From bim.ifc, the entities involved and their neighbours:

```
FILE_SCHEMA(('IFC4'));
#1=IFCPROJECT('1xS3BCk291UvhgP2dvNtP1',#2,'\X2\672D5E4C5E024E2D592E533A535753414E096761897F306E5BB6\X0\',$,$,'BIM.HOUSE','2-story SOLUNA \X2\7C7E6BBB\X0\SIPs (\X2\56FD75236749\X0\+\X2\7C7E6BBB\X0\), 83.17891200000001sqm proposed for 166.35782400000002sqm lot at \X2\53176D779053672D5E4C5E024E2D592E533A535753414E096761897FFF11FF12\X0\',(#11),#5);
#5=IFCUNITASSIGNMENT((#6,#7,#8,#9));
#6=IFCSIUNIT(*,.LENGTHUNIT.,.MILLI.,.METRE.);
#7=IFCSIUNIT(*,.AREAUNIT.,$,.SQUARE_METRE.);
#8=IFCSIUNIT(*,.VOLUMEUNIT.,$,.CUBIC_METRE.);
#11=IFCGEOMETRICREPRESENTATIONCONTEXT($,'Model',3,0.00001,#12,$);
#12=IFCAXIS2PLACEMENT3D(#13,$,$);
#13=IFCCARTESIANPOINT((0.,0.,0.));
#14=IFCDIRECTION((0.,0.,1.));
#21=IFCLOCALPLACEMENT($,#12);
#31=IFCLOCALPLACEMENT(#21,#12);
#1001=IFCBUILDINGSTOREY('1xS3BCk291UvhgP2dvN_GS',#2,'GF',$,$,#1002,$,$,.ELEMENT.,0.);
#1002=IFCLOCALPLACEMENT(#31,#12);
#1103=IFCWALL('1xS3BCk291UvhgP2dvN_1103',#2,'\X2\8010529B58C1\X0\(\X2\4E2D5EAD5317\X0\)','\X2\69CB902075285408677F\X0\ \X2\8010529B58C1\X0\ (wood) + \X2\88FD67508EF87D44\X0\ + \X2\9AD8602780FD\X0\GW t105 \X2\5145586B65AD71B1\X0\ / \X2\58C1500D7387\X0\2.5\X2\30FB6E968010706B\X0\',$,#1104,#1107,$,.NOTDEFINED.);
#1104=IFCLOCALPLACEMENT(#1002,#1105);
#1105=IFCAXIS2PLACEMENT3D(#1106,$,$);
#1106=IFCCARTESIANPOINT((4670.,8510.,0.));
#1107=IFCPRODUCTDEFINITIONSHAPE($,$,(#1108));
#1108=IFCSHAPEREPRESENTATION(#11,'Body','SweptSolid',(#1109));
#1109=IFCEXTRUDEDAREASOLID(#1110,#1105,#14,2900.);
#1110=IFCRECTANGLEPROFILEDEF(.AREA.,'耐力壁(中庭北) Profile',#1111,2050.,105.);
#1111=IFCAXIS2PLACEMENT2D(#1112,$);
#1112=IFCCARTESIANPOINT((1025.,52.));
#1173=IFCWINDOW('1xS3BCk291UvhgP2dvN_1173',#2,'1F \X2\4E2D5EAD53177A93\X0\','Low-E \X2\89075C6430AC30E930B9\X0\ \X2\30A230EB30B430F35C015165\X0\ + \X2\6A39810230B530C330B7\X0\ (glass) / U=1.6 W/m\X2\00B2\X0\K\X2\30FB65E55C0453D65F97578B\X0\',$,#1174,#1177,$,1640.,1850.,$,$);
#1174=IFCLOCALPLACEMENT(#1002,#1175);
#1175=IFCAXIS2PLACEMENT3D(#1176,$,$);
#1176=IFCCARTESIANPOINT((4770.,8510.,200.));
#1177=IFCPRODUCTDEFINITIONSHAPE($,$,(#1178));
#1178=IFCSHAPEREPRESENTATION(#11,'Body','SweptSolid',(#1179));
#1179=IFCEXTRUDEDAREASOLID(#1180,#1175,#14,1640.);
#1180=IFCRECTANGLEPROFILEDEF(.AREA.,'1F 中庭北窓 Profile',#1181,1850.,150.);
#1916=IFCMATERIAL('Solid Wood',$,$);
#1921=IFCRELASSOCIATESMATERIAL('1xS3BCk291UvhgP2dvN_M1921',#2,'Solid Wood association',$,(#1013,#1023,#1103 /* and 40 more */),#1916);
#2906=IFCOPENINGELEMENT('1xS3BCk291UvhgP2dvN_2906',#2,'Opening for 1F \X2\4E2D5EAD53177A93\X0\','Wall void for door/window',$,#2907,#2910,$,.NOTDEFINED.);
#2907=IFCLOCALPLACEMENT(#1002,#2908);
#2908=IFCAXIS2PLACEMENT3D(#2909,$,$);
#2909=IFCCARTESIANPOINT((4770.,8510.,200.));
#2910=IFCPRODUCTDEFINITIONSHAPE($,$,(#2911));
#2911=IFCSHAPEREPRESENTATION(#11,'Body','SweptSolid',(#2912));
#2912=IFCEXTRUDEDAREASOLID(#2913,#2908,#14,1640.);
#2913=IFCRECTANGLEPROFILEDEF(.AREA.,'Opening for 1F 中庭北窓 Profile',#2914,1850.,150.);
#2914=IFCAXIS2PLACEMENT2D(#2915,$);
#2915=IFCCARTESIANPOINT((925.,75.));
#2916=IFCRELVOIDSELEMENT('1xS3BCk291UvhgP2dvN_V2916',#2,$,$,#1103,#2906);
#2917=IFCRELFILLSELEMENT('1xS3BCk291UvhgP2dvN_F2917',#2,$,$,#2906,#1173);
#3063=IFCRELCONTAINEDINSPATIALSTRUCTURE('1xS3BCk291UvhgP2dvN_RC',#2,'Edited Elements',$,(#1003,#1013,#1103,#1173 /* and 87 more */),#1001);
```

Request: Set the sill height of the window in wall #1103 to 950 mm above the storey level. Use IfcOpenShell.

```python
import numpy as np
import ifcopenshell
import ifcopenshell.api.geometry
import ifcopenshell.geom
import ifcopenshell.util.element
import ifcopenshell.util.placement
import ifcopenshell.util.shape
import ifcopenshell.util.unit

model = ifcopenshell.open("bim.ifc")
unit_scale = ifcopenshell.util.unit.calculate_unit_scale(model)

window = model.by_id(1173)
opening = window.FillsVoids[0].RelatingOpeningElement
storey = ifcopenshell.util.element.get_container(window, ifc_class="IfcBuildingStorey")
level = ifcopenshell.util.placement.get_local_placement(storey.ObjectPlacement)[2, 3]

# The opening's origin need not be at the sill, so measure its lowest point.
shape = ifcopenshell.geom.create_shape(ifcopenshell.geom.settings(), opening)
bottom = ifcopenshell.util.shape.get_shape_bottom_elevation(shape, shape.geometry) / unit_scale
dz = level + 0.95 / unit_scale - bottom

shift = np.array([0.0, 0.0, dz])
# The window is not placed relative to its opening, so move both.
for product in (opening, window):
    matrix = ifcopenshell.util.placement.get_local_placement(product.ObjectPlacement)
    matrix[:3, 3] += shift
    ifcopenshell.api.geometry.edit_object_placement(model, product=product, matrix=matrix, is_si=False)

print(f"moved by {dz * unit_scale:+.3f} m")

model.write("bim_updated.ifc")
```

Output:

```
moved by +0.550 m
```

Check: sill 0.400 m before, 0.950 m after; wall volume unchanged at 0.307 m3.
